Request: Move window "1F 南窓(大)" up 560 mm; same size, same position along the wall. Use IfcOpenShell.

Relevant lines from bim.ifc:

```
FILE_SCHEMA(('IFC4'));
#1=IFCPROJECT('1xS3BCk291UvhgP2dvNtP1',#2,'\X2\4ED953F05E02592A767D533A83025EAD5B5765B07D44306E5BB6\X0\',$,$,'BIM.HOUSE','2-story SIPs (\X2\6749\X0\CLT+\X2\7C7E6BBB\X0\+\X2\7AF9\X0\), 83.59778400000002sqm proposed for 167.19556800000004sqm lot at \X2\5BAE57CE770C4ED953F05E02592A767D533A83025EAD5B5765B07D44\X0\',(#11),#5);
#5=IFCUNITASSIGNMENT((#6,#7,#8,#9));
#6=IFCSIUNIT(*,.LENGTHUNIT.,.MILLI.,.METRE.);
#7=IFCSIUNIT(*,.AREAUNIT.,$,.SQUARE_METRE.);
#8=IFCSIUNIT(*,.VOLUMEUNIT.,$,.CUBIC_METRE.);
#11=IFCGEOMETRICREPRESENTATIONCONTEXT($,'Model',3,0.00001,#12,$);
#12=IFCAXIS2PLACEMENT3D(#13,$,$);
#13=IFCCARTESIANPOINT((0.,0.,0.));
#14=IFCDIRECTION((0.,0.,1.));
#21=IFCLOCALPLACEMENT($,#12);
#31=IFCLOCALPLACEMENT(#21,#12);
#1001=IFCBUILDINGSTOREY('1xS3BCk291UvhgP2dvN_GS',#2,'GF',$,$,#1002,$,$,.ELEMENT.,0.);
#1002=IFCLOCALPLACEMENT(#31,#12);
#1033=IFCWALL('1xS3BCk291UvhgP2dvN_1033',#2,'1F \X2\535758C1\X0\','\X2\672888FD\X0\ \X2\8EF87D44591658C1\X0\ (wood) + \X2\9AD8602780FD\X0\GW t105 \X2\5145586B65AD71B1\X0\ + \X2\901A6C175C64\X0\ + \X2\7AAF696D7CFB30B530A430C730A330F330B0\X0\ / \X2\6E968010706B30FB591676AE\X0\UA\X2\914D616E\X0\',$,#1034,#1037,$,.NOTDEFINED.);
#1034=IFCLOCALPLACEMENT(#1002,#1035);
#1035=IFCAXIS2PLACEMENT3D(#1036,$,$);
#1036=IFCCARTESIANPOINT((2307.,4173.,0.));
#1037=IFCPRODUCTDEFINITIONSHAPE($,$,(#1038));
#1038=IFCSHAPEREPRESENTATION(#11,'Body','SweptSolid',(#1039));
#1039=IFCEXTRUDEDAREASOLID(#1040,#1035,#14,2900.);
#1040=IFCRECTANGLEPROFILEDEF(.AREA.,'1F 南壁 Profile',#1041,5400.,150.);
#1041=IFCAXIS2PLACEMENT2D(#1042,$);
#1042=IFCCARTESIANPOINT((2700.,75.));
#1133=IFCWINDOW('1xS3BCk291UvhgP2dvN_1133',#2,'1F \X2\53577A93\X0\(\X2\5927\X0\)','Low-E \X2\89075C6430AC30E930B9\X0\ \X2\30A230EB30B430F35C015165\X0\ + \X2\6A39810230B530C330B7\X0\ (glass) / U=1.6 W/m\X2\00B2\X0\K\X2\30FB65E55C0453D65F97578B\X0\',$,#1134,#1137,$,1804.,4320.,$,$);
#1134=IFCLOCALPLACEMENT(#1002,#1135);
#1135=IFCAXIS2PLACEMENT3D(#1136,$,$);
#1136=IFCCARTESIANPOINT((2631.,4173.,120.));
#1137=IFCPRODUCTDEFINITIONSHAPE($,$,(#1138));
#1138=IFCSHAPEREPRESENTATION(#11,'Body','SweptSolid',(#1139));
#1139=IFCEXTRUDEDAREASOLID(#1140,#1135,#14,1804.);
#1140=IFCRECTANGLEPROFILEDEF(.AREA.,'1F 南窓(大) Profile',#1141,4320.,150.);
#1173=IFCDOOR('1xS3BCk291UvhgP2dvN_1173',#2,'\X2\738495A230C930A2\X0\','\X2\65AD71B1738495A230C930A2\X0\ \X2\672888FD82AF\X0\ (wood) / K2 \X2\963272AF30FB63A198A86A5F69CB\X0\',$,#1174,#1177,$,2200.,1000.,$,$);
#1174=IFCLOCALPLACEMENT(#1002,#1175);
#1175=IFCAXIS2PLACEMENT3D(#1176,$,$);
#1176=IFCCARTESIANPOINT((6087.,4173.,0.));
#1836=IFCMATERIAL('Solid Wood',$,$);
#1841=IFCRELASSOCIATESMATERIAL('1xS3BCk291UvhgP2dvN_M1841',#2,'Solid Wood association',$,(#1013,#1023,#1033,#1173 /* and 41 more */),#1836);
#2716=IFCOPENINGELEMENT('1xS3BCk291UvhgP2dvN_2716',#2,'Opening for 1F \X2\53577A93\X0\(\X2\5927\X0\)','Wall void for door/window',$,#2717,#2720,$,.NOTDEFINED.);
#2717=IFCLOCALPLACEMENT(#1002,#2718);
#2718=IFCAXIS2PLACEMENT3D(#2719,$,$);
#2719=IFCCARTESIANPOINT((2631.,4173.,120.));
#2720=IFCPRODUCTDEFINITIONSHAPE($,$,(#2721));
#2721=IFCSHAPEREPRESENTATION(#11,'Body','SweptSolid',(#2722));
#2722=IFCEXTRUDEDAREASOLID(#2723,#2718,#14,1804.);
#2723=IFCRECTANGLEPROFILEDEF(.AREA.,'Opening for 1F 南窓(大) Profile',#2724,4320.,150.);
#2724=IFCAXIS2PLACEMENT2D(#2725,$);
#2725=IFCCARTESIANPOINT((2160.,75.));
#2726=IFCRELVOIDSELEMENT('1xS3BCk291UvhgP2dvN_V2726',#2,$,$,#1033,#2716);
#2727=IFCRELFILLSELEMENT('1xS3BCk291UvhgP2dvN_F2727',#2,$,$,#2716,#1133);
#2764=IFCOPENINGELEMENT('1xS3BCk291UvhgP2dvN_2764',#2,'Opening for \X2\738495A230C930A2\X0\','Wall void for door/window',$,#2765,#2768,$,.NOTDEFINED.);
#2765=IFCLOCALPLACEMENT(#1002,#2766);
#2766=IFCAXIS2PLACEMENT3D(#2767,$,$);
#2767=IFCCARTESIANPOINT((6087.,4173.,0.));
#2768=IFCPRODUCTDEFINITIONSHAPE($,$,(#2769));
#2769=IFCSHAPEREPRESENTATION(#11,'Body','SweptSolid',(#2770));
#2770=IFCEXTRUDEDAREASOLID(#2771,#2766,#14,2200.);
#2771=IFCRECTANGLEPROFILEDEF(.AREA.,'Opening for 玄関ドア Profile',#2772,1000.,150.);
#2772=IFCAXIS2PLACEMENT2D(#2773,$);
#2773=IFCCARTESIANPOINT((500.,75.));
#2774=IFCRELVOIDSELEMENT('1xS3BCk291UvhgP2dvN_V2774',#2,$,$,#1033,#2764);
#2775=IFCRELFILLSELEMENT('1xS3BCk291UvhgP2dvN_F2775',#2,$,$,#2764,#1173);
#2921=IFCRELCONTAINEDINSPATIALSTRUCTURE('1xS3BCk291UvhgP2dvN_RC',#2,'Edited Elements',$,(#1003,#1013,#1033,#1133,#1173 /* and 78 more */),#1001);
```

```python
import numpy as np
import ifcopenshell
import ifcopenshell.api.geometry
import ifcopenshell.util.placement
import ifcopenshell.util.unit

model = ifcopenshell.open("bim.ifc")
unit_scale = ifcopenshell.util.unit.calculate_unit_scale(model)

window = model.by_id(1133)
opening = window.FillsVoids[0].RelatingOpeningElement
dz = 560.0

shift = np.array([0.0, 0.0, dz])
# The window is not placed relative to its opening, so move both.
for product in (opening, window):
    matrix = ifcopenshell.util.placement.get_local_placement(product.ObjectPlacement)
    matrix[:3, 3] += shift
    ifcopenshell.api.geometry.edit_object_placement(model, product=product, matrix=matrix, is_si=False)

print(f"moved by {dz * unit_scale:+.3f} m")

model.write("bim_rev.ifc")
```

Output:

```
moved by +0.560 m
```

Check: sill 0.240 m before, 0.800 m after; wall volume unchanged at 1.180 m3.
